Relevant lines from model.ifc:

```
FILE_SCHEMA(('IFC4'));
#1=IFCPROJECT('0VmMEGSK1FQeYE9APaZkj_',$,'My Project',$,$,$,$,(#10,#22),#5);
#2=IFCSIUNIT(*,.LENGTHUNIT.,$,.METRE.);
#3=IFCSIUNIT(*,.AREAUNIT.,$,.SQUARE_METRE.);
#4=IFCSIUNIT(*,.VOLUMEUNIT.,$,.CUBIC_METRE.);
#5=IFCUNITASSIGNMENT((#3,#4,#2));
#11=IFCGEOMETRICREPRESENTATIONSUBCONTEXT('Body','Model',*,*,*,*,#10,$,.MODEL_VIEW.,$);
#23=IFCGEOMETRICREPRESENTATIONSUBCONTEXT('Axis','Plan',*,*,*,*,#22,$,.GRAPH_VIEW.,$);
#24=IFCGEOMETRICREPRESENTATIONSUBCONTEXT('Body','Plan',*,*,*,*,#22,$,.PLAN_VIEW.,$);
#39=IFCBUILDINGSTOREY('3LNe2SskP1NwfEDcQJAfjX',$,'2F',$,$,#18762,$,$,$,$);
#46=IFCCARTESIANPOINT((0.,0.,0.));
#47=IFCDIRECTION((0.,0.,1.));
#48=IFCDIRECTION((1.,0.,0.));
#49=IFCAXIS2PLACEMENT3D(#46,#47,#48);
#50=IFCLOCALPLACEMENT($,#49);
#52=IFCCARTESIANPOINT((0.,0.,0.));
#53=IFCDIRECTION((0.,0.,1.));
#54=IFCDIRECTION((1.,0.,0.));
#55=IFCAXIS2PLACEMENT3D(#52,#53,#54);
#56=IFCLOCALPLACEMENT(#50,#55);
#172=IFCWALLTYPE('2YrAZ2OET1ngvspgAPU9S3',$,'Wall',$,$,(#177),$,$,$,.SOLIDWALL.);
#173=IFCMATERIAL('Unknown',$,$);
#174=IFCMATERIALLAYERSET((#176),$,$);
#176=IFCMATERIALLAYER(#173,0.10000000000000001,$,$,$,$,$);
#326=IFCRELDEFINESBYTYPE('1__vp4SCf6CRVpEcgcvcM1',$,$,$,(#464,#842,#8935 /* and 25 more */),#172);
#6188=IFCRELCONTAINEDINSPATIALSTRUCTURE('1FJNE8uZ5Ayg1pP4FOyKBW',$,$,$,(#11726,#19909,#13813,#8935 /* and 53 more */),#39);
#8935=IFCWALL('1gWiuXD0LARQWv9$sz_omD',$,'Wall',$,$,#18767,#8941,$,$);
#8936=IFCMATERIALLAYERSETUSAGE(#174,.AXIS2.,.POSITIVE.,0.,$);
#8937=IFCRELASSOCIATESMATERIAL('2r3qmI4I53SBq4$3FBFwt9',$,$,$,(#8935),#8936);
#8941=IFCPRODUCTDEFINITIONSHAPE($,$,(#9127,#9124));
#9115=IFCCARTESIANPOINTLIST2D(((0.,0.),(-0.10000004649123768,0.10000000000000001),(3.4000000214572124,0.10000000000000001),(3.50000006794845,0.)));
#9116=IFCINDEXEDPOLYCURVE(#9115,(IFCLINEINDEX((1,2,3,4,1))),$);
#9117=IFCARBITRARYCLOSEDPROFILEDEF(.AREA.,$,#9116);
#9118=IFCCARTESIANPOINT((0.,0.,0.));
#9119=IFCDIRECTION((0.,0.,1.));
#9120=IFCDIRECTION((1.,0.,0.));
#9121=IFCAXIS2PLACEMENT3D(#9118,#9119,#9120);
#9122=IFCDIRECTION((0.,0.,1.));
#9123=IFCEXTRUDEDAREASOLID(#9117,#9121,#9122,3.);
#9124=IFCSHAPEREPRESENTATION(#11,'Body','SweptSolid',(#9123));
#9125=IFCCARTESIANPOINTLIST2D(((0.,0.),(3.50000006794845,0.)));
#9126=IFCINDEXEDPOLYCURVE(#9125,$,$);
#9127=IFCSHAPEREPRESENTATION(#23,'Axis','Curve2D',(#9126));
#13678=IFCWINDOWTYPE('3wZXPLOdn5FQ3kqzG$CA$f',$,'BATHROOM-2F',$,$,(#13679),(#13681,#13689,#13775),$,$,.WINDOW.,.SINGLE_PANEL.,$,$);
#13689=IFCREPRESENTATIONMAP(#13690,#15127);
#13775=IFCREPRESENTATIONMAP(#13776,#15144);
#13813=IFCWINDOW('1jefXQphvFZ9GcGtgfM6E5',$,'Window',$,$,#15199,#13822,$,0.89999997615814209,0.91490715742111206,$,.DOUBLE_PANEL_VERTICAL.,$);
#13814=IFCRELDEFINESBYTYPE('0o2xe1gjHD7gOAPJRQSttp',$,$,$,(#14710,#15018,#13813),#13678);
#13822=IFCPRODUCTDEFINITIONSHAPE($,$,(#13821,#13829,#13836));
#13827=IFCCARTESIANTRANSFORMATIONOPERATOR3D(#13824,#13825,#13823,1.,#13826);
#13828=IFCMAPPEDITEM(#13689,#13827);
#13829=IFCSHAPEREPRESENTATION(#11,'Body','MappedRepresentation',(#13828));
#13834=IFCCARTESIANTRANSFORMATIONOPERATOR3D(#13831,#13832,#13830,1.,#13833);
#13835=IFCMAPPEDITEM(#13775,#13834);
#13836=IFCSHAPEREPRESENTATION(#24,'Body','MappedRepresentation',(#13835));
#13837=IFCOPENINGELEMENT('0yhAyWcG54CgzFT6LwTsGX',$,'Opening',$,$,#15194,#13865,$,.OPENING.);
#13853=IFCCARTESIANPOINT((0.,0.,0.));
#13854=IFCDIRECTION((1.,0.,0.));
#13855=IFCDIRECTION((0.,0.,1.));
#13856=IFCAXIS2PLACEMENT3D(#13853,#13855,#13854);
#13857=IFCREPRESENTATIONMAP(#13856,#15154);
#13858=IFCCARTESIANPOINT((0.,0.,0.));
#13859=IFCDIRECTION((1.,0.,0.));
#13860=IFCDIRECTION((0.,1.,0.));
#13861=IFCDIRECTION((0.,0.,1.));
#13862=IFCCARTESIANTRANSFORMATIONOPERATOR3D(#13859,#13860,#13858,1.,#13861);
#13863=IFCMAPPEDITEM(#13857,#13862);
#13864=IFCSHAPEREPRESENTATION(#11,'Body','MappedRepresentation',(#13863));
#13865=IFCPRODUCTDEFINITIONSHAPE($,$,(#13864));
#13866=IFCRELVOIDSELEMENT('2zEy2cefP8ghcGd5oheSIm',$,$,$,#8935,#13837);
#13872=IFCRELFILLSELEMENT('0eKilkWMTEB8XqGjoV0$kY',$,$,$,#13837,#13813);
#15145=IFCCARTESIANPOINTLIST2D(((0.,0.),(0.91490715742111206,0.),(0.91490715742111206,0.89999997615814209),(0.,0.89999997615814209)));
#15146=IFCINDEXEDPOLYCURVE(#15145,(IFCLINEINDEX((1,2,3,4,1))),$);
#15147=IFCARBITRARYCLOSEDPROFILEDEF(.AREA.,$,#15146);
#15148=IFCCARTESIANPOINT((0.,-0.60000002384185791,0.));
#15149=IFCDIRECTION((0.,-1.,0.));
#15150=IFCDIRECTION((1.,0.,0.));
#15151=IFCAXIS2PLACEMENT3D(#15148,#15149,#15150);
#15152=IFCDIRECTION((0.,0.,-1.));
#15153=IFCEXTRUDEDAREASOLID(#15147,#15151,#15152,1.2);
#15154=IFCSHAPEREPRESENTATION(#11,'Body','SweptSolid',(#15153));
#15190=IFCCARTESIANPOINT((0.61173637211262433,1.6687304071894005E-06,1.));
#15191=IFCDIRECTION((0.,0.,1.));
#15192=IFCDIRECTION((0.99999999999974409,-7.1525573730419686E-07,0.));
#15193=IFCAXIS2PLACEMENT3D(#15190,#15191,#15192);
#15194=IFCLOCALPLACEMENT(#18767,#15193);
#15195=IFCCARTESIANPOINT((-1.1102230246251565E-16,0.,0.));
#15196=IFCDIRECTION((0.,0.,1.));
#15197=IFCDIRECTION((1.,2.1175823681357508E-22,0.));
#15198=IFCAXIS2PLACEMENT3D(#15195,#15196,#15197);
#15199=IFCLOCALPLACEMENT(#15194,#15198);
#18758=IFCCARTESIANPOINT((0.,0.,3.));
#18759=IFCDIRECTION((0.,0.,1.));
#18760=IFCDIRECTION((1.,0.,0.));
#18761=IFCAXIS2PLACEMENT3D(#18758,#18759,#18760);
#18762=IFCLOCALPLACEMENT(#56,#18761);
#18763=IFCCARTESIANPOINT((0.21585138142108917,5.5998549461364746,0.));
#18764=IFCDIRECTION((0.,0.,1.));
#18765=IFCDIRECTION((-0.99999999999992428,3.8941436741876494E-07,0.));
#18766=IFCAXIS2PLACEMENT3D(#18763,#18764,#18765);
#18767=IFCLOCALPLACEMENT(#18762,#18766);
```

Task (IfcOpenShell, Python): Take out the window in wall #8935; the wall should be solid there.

```python
import ifcopenshell
import ifcopenshell.api.feature
import ifcopenshell.api.root
import ifcopenshell.geom
import ifcopenshell.util.shape

model = ifcopenshell.open("model.ifc")
settings = ifcopenshell.geom.settings()


def volume(element):
    """Net volume in cubic metres, openings subtracted."""
    shape = ifcopenshell.geom.create_shape(settings, element)
    return ifcopenshell.util.shape.get_volume(shape.geometry)


window = model.by_id(13813)
opening = window.FillsVoids[0].RelatingOpeningElement
wall = opening.VoidsElements[0].RelatingBuildingElement
before = volume(wall)

ifcopenshell.api.root.remove_product(model, product=window)
ifcopenshell.api.feature.remove_feature(model, feature=opening)

after = volume(wall)

print(f"wall volume {before:.3f} -> {after:.3f} m3")

model.write("model_rev.ifc")
```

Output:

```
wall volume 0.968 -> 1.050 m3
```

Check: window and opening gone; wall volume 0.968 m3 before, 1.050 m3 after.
